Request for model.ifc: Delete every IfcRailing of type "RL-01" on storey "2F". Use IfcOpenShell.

First a look at what the model holds.

```python
import ifcopenshell
import ifcopenshell.util.element

model = ifcopenshell.open("model.ifc")
print(model.schema)
storey = next(s for s in model.by_type("IfcBuildingStorey") if s.Name == "2F")
railings = [e for e in ifcopenshell.util.element.get_decomposition(storey) if e.is_a("IfcRailing")]
seen = {}
for e in railings:
    element_type = ifcopenshell.util.element.get_type(e)
    name = element_type.Name if element_type not in (None, e) else None
    seen[name] = seen.get(name, 0) + 1
for name, count in sorted(seen.items(), key=str):
    print(count, "x", name)
```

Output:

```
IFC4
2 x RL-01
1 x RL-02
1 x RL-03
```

```python
import ifcopenshell
import ifcopenshell.api.root
import ifcopenshell.util.element

model = ifcopenshell.open("model.ifc")

storey = next(s for s in model.by_type("IfcBuildingStorey") if s.Name == "2F")
railings = [e for e in ifcopenshell.util.element.get_decomposition(storey) if e.is_a("IfcRailing")]
targets = [e for e in railings if (t := ifcopenshell.util.element.get_type(e)) not in (None, e) and t.Name == "RL-01"]

for e in targets:
    ifcopenshell.api.root.remove_product(model, product=e)
print(len(targets), "removed")

model.write("model_updated.ifc")
```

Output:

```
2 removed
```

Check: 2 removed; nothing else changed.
